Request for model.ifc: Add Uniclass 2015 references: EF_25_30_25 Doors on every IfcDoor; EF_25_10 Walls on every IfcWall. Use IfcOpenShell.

First a look at what the model holds.

```python
import ifcopenshell

model = ifcopenshell.open("model.ifc")
print(model.schema)
print("classifications:", [c.Name for c in model.by_type("IfcClassification")])
for ifc_class in ("IfcDoor", "IfcRoof", "IfcStair", "IfcWall", "IfcWindow"):
    print(ifc_class, len(model.by_type(ifc_class)))
```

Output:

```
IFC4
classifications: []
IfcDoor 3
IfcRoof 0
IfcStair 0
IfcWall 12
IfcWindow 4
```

```python
import ifcopenshell
import ifcopenshell.api.classification

model = ifcopenshell.open("model.ifc")

system = ifcopenshell.api.classification.add_classification(model, classification="Uniclass 2015")

codes = {
    "IfcDoor": ("EF_25_30_25", "Doors"),
    "IfcWall": ("EF_25_10", "Walls"),
}
for ifc_class, (code, name) in codes.items():
    products = model.by_type(ifc_class)
    ifcopenshell.api.classification.add_reference(
        model, products=products, classification=system, identification=code, name=name
    )
    print(code, len(products))

model.write("model_rev.ifc")
```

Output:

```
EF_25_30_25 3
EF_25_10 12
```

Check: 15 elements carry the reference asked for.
